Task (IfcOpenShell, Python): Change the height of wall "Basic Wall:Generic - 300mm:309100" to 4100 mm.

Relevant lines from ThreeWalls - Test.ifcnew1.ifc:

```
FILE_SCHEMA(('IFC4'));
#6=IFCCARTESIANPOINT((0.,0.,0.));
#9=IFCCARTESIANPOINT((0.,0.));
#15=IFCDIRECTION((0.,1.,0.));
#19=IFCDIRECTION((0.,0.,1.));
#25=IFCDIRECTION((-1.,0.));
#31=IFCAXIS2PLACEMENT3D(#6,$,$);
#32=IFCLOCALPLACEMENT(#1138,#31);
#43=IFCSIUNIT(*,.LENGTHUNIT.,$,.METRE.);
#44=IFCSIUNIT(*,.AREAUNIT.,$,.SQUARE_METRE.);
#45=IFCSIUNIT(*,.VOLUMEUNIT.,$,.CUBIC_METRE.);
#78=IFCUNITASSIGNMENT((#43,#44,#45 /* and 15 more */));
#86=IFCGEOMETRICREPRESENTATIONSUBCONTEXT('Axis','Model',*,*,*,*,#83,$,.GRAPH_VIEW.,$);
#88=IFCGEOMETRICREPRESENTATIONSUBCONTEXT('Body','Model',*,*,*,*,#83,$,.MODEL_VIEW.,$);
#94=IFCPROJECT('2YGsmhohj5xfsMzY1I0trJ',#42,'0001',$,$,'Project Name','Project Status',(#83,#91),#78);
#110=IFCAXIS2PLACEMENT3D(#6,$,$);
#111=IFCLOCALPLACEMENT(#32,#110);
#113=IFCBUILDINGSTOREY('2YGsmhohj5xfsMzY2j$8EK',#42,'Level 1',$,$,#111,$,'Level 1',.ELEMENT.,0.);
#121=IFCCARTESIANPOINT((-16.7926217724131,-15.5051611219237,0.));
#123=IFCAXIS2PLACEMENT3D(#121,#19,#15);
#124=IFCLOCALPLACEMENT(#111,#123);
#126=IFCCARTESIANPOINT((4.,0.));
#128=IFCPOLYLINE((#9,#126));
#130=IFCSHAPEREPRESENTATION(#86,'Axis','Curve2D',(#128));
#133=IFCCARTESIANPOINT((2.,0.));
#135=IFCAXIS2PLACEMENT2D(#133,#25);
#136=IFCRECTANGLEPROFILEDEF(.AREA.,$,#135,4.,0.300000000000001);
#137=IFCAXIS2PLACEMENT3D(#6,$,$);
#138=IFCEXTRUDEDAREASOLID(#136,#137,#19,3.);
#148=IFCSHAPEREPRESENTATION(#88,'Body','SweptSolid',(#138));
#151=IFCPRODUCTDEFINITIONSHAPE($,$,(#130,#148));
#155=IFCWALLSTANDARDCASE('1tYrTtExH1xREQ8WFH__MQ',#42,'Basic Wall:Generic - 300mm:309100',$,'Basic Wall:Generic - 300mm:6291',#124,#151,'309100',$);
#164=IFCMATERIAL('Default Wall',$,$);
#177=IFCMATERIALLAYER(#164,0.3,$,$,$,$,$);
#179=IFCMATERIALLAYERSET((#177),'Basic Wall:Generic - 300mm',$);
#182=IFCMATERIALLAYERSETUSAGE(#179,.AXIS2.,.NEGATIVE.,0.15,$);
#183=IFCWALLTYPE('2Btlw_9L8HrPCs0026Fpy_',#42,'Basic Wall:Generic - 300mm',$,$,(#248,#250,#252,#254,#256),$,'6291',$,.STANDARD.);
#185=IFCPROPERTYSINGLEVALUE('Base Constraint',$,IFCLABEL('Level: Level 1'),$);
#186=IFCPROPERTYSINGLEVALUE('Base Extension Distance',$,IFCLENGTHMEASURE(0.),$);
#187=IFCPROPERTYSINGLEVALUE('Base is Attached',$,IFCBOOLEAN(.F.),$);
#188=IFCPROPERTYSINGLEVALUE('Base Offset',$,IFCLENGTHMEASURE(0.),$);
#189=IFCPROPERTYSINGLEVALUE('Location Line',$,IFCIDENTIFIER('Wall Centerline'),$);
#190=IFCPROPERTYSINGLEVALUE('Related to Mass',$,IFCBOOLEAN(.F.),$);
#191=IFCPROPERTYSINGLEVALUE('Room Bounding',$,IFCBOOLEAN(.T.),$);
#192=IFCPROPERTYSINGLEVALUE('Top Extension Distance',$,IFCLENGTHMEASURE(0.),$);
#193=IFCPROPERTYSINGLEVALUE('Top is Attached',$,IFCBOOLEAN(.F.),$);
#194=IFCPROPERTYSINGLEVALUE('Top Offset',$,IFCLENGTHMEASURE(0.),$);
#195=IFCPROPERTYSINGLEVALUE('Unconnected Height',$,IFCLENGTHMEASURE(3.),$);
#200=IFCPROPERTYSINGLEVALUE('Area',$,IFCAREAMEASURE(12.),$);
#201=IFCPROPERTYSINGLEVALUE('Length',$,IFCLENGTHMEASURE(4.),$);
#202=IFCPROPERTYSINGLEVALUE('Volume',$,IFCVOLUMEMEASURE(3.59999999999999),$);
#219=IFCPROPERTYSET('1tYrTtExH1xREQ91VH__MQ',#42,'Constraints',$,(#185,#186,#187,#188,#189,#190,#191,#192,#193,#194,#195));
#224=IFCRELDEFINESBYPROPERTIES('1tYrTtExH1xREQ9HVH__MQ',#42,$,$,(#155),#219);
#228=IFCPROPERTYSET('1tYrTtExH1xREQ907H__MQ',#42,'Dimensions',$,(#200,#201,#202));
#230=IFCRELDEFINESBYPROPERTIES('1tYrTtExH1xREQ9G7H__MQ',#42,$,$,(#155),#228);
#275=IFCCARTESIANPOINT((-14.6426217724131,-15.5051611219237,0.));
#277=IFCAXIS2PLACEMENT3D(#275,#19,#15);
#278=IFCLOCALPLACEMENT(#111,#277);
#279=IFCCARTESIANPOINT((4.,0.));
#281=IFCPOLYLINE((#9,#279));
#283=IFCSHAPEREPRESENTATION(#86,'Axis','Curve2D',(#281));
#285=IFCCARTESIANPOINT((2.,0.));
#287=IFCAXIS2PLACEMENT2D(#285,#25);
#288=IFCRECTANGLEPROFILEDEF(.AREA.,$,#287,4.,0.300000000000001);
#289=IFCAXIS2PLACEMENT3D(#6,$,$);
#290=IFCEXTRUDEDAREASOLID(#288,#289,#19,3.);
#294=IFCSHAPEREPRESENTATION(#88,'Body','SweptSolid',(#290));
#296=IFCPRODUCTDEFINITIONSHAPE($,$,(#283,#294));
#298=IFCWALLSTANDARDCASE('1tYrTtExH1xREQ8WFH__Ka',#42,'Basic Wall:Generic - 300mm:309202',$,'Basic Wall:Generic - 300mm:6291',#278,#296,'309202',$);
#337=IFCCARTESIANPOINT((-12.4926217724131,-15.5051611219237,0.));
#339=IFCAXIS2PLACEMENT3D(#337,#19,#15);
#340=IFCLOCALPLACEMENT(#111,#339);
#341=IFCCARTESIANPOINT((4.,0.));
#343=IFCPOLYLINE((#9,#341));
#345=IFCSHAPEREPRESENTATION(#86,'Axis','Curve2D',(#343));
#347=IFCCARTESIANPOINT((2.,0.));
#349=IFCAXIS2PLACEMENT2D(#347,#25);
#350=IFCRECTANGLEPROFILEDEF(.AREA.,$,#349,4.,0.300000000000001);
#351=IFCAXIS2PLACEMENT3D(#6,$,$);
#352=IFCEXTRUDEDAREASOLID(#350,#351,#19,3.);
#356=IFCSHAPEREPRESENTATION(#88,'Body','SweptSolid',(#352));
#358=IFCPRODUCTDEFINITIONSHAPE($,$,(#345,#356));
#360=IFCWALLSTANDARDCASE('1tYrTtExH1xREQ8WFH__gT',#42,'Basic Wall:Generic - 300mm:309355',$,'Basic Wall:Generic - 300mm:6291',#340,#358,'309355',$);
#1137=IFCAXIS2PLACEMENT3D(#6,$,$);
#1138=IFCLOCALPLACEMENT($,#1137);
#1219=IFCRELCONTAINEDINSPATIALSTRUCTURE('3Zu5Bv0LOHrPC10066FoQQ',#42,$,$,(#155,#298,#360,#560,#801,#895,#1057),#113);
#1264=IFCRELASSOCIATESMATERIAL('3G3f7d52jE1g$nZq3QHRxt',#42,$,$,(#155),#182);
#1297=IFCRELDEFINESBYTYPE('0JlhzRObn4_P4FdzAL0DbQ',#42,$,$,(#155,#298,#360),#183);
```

```python
import ifcopenshell
import ifcopenshell.api.pset
import ifcopenshell.geom
import ifcopenshell.util.element
import ifcopenshell.util.representation
import ifcopenshell.util.shape
import ifcopenshell.util.unit

model = ifcopenshell.open("ThreeWalls - Test.ifcnew1.ifc")
unit_scale = ifcopenshell.util.unit.calculate_unit_scale(model)
area_scale = ifcopenshell.util.unit.calculate_unit_scale(model, "AREAUNIT")
volume_scale = ifcopenshell.util.unit.calculate_unit_scale(model, "VOLUMEUNIT")
settings = ifcopenshell.geom.settings()


def volume(element):
    """Net volume in cubic metres, openings subtracted."""
    shape = ifcopenshell.geom.create_shape(settings, element)
    return ifcopenshell.util.shape.get_volume(shape.geometry)


wall = model.by_guid("1tYrTtExH1xREQ8WFH__MQ")
before = volume(wall)

body = ifcopenshell.util.representation.get_representation(wall, "Model", "Body")
solid = body.Items[0]
old_height = solid.Depth
solid.Depth = 4.1 / unit_scale
after = volume(wall)
thickness = 0.3  # wall thickness in metres

# Update the stored height, areas and volumes.
pset = model.by_id(ifcopenshell.util.element.get_pset(wall, "Constraints", should_inherit=False)["id"])
ifcopenshell.api.pset.edit_pset(model, pset=pset, properties={
    "Unconnected Height": model.create_entity("IfcLengthMeasure", solid.Depth),
})
pset = model.by_id(ifcopenshell.util.element.get_pset(wall, "Dimensions", should_inherit=False)["id"])
ifcopenshell.api.pset.edit_pset(model, pset=pset, properties={
    "Area": model.create_entity("IfcAreaMeasure", after / thickness / area_scale),
    "Volume": model.create_entity("IfcVolumeMeasure", after / volume_scale),
})

print(f"height {old_height:g} -> {solid.Depth:g}, volume {before:.3f} -> {after:.3f} m3")

model.write("ThreeWalls - Test.ifcnew1-out.ifc")
```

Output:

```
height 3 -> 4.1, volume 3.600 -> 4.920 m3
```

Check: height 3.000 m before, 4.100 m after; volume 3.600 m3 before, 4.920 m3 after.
